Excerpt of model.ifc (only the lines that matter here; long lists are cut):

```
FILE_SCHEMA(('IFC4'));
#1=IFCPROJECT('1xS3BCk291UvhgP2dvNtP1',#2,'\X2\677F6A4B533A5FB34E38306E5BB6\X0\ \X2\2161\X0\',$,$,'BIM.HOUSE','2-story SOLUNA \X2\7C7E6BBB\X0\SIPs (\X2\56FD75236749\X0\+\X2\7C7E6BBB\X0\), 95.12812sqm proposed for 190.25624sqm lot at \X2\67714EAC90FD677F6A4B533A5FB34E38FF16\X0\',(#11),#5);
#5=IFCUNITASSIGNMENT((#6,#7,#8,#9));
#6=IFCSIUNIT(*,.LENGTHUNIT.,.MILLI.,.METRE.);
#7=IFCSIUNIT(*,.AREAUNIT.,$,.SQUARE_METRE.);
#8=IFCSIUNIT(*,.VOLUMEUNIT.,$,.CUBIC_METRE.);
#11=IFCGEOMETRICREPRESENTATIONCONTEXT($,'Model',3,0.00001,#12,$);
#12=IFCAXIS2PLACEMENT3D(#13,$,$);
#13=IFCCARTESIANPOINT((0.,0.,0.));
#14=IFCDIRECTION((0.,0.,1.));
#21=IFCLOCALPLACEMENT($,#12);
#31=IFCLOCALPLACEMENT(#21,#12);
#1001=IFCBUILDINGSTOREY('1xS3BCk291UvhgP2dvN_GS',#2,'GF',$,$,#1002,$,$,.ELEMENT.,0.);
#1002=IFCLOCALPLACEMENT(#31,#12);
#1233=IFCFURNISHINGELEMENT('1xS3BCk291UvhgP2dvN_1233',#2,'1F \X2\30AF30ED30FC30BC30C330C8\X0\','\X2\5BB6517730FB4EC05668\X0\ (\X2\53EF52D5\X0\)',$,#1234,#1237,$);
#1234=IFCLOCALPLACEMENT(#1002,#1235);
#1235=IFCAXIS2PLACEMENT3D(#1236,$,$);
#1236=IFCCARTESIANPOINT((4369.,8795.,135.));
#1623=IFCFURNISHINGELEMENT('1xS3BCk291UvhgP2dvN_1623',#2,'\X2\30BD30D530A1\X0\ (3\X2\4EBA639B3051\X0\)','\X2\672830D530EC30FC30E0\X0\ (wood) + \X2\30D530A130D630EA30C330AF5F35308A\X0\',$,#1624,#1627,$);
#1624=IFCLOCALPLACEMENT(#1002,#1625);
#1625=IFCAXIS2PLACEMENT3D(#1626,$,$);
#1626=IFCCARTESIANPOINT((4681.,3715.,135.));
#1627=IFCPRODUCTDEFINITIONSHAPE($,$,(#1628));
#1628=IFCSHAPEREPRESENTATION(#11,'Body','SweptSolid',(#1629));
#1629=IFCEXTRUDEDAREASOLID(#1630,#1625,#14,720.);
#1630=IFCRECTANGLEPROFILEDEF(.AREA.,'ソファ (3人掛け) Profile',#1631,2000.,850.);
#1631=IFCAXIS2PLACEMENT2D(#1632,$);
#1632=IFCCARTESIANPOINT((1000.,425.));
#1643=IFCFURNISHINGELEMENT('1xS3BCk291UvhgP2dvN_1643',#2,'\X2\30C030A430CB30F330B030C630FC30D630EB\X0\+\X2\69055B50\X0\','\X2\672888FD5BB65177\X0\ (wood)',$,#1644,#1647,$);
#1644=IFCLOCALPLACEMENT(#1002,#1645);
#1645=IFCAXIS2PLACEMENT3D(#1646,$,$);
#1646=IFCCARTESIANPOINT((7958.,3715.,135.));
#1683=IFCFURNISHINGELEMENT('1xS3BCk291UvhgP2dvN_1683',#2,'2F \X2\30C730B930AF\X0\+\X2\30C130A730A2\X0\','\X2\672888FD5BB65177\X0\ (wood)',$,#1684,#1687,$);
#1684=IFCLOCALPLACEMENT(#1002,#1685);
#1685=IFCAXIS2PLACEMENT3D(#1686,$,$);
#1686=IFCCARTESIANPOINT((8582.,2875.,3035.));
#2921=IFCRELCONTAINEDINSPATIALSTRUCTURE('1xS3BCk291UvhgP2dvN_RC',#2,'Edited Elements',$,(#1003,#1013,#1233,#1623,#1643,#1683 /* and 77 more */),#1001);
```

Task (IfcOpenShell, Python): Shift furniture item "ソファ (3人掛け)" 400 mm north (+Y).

```python
import ifcopenshell
import ifcopenshell.api.geometry
import ifcopenshell.util.placement
import ifcopenshell.util.unit

model = ifcopenshell.open("model.ifc")
unit_scale = ifcopenshell.util.unit.calculate_unit_scale(model)

item = model.by_guid("1xS3BCk291UvhgP2dvN_1623")
matrix = ifcopenshell.util.placement.get_local_placement(item.ObjectPlacement)
matrix[1, 3] += 0.4 / unit_scale
ifcopenshell.api.geometry.edit_object_placement(model, product=item, matrix=matrix, is_si=False)

print(ifcopenshell.util.placement.get_local_placement(item.ObjectPlacement).round(3) + 0.0)

model.write("model_rev.ifc")
```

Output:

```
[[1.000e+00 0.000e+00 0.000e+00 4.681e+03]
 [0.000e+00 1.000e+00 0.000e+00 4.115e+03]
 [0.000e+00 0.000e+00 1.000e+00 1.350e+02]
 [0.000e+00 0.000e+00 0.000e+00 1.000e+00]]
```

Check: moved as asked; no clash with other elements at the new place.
